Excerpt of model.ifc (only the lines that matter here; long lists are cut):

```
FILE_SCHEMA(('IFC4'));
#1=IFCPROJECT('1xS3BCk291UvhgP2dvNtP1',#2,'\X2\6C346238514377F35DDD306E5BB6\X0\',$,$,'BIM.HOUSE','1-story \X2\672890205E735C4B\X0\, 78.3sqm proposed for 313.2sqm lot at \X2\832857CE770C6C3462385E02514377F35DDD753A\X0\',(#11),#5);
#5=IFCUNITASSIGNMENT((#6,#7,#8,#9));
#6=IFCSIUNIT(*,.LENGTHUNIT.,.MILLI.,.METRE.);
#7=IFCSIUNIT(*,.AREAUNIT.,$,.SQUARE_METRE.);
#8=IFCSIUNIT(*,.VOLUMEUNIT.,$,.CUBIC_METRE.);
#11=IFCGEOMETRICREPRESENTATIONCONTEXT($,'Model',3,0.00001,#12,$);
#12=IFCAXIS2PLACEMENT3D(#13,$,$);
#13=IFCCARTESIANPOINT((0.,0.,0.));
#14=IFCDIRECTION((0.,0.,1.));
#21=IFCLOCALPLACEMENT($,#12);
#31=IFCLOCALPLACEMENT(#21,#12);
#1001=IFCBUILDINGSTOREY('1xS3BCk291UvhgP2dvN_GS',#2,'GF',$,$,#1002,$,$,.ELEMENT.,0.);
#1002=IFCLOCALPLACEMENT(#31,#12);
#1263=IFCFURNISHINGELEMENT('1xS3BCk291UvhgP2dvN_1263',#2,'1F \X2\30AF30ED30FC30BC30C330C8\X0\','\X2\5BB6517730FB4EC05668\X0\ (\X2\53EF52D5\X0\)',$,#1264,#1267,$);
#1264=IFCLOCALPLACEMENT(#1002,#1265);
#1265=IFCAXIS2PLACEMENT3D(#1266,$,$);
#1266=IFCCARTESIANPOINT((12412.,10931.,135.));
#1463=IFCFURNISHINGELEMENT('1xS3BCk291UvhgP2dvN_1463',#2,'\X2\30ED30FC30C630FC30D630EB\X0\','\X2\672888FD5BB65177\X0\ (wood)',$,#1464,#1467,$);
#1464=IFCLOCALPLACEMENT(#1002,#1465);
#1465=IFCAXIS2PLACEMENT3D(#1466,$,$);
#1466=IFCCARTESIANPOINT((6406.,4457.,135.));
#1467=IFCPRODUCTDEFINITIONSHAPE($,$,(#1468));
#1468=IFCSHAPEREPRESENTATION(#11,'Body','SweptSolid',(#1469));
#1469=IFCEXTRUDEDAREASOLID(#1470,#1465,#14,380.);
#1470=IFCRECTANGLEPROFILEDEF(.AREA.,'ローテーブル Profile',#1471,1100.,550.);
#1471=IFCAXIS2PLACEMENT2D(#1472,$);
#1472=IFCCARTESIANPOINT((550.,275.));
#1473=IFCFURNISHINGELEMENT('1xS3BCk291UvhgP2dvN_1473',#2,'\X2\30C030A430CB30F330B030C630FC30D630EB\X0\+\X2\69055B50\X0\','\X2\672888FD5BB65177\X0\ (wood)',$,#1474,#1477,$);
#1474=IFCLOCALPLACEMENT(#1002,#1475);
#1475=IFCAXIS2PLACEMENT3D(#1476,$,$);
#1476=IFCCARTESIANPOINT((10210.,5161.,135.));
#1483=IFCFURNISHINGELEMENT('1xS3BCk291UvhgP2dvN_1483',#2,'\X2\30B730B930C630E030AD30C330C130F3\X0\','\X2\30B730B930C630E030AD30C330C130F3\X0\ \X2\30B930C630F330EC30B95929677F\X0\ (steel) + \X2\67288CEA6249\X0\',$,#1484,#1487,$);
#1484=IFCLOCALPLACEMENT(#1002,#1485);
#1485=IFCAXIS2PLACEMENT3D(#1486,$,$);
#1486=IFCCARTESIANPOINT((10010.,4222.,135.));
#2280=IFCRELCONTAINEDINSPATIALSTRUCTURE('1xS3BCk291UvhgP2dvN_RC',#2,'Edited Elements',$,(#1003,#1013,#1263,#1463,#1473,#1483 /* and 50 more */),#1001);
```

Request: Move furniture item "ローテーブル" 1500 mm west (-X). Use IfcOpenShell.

```python
import ifcopenshell
import ifcopenshell.api.geometry
import ifcopenshell.util.placement

model = ifcopenshell.open("model.ifc")

item = model.by_guid("1xS3BCk291UvhgP2dvN_1463")
matrix = ifcopenshell.util.placement.get_local_placement(item.ObjectPlacement)
matrix[0, 3] -= 1500.0
ifcopenshell.api.geometry.edit_object_placement(model, product=item, matrix=matrix, is_si=False)

print(ifcopenshell.util.placement.get_local_placement(item.ObjectPlacement).round(3) + 0.0)

model.write("model_v2.ifc")
```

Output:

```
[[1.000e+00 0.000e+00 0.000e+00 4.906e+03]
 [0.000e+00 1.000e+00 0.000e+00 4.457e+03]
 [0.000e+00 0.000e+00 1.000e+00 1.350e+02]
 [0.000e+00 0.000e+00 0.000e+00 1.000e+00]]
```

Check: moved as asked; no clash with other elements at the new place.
